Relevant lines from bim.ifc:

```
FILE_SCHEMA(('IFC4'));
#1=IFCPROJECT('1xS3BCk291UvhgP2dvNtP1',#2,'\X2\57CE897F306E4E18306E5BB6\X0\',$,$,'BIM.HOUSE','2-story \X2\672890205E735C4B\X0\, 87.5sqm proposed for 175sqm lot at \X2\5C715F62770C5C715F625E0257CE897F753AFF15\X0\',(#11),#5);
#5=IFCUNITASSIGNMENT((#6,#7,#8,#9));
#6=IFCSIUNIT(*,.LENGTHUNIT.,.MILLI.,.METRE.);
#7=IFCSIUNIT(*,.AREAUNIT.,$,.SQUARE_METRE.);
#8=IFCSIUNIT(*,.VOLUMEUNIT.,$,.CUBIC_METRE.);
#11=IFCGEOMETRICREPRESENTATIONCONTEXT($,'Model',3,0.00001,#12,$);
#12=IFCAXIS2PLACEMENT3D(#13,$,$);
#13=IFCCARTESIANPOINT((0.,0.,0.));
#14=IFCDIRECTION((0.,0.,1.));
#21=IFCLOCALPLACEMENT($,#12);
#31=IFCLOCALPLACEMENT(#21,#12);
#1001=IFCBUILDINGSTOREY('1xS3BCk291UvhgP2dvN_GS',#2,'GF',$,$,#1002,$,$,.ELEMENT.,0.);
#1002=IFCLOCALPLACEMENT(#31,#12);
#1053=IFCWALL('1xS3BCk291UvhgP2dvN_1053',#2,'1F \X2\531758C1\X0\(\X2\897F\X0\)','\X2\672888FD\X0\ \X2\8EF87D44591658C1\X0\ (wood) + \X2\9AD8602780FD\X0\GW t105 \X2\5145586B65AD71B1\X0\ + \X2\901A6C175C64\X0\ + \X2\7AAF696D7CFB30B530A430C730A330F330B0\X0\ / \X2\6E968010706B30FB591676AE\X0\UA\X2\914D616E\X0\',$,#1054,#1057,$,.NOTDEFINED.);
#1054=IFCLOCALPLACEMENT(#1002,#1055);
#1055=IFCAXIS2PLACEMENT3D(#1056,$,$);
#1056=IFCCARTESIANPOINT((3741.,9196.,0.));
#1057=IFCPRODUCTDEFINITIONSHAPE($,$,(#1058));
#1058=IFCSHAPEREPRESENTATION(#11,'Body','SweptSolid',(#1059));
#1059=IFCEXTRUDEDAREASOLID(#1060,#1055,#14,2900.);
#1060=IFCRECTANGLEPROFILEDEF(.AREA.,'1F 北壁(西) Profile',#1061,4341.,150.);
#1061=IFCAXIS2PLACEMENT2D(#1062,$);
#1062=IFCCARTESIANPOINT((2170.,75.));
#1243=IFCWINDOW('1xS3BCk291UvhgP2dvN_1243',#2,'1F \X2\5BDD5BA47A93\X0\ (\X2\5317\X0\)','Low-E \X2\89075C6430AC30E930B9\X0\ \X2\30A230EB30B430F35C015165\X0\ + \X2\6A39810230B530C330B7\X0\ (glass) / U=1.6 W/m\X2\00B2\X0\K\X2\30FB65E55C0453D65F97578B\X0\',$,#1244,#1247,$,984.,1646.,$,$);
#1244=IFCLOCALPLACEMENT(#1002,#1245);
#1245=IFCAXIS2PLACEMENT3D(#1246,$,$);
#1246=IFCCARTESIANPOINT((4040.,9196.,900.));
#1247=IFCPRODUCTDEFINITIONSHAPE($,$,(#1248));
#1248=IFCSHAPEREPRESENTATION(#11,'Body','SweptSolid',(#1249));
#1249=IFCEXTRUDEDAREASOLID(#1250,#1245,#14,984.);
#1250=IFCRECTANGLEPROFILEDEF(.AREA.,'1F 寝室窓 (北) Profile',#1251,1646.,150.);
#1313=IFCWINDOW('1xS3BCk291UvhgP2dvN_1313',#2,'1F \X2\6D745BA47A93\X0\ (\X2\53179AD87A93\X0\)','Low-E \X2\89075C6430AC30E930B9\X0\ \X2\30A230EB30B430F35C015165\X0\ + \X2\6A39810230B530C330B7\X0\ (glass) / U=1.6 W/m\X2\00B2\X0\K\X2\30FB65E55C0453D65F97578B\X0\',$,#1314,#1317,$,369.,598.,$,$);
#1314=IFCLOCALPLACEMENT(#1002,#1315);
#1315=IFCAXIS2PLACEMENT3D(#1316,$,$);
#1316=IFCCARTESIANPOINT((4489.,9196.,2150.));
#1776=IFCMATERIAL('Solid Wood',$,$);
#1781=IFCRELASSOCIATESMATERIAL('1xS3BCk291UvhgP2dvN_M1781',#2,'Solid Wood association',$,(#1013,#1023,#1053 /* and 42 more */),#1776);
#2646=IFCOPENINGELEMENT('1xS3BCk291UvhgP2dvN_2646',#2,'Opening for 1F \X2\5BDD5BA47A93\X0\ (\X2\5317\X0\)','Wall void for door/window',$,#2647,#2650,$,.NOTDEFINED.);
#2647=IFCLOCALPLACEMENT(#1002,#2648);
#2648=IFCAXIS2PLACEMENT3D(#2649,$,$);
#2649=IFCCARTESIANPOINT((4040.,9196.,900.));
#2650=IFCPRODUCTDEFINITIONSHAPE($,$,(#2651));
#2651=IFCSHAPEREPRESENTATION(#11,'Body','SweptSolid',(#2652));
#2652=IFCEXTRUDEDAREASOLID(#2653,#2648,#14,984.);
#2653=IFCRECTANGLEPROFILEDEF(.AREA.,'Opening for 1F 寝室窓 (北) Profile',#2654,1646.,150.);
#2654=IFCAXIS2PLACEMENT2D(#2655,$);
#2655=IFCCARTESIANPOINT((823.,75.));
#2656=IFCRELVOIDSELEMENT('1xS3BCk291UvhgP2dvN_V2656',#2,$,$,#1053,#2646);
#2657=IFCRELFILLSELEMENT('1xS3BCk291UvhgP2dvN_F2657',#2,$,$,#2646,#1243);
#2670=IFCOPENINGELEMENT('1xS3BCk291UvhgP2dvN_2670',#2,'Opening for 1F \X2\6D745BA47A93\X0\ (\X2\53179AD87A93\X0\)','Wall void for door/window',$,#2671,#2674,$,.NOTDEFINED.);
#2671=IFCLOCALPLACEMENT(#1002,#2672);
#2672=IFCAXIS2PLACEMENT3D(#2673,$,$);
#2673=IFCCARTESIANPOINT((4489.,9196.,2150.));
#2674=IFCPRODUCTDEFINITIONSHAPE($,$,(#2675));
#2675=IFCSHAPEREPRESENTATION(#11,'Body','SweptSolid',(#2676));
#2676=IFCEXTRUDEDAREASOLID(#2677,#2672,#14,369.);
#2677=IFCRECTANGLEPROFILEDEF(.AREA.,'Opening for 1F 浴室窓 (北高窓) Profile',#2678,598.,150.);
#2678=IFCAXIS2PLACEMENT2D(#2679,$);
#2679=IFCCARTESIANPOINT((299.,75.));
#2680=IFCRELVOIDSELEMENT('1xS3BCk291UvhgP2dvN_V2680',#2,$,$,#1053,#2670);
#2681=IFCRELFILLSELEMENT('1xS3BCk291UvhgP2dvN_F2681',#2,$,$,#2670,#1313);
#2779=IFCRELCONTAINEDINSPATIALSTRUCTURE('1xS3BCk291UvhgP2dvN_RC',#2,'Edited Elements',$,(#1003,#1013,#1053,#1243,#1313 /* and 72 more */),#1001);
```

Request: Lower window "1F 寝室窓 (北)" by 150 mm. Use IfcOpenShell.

```python
import numpy as np
import ifcopenshell
import ifcopenshell.api.geometry
import ifcopenshell.util.placement
import ifcopenshell.util.unit

model = ifcopenshell.open("bim.ifc")
unit_scale = ifcopenshell.util.unit.calculate_unit_scale(model)

window = model.by_guid("1xS3BCk291UvhgP2dvN_1243")
opening = window.FillsVoids[0].RelatingOpeningElement
dz = -0.15 / unit_scale

shift = np.array([0.0, 0.0, dz])
# The window is not placed relative to its opening, so move both.
for product in (opening, window):
    matrix = ifcopenshell.util.placement.get_local_placement(product.ObjectPlacement)
    matrix[:3, 3] += shift
    ifcopenshell.api.geometry.edit_object_placement(model, product=product, matrix=matrix, is_si=False)

print(f"moved by {dz * unit_scale:+.3f} m")

model.write("bim_rev.ifc")
```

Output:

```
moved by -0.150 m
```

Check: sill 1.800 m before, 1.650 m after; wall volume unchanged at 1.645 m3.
